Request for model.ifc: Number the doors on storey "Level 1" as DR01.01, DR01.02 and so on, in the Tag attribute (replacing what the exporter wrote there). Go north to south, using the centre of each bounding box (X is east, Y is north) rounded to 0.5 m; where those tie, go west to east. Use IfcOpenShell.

First a look at what the model holds.

```python
import ifcopenshell
import ifcopenshell.util.element
import ifcopenshell.util.placement

model = ifcopenshell.open("model.ifc")
print(model.schema)
storey = next(s for s in model.by_type("IfcBuildingStorey") if s.Name == "Level 1")
doors = [e for e in ifcopenshell.util.element.get_decomposition(storey) if e.is_a("IfcDoor")]
for e in sorted(doors, key=lambda e: e.id()):
    origin = ifcopenshell.util.placement.get_local_placement(e.ObjectPlacement)[:3, 3]
    print(e.id(), e.Tag, e.Name, origin.round(2) + 0.0, sep=" | ")
```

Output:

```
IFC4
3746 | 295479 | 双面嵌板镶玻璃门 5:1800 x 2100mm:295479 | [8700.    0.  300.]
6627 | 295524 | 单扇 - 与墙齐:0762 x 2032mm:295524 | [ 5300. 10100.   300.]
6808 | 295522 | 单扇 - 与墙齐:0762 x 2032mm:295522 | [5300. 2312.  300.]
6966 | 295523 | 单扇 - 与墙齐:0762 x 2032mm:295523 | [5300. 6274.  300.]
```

```python
import ifcopenshell
import ifcopenshell.geom
import ifcopenshell.util.element
import ifcopenshell.util.shape

model = ifcopenshell.open("model.ifc")
settings = ifcopenshell.geom.settings()
settings.set("use-world-coords", True)


def centre(element):
    shape = ifcopenshell.geom.create_shape(settings, element)
    return ifcopenshell.util.shape.get_bbox_centroid(shape.geometry)


storey = next(s for s in model.by_type("IfcBuildingStorey") if s.Name == "Level 1")
doors = [e for e in ifcopenshell.util.element.get_decomposition(storey) if e.is_a("IfcDoor")]

# Insertion points can sit at a corner or the storey origin, so sort by the geometry (in metres).
centres = {e: centre(e) for e in doors}
doors.sort(key=lambda e: (-round(centres[e][1] / 0.5), centres[e][0]))

for i, e in enumerate(doors, start=1):
    number = f"DR01.{i:02d}"
    e.Tag = number
    print(e.id(), number)

model.write("model-out.ifc")
```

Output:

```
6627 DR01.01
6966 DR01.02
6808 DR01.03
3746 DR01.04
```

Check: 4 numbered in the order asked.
